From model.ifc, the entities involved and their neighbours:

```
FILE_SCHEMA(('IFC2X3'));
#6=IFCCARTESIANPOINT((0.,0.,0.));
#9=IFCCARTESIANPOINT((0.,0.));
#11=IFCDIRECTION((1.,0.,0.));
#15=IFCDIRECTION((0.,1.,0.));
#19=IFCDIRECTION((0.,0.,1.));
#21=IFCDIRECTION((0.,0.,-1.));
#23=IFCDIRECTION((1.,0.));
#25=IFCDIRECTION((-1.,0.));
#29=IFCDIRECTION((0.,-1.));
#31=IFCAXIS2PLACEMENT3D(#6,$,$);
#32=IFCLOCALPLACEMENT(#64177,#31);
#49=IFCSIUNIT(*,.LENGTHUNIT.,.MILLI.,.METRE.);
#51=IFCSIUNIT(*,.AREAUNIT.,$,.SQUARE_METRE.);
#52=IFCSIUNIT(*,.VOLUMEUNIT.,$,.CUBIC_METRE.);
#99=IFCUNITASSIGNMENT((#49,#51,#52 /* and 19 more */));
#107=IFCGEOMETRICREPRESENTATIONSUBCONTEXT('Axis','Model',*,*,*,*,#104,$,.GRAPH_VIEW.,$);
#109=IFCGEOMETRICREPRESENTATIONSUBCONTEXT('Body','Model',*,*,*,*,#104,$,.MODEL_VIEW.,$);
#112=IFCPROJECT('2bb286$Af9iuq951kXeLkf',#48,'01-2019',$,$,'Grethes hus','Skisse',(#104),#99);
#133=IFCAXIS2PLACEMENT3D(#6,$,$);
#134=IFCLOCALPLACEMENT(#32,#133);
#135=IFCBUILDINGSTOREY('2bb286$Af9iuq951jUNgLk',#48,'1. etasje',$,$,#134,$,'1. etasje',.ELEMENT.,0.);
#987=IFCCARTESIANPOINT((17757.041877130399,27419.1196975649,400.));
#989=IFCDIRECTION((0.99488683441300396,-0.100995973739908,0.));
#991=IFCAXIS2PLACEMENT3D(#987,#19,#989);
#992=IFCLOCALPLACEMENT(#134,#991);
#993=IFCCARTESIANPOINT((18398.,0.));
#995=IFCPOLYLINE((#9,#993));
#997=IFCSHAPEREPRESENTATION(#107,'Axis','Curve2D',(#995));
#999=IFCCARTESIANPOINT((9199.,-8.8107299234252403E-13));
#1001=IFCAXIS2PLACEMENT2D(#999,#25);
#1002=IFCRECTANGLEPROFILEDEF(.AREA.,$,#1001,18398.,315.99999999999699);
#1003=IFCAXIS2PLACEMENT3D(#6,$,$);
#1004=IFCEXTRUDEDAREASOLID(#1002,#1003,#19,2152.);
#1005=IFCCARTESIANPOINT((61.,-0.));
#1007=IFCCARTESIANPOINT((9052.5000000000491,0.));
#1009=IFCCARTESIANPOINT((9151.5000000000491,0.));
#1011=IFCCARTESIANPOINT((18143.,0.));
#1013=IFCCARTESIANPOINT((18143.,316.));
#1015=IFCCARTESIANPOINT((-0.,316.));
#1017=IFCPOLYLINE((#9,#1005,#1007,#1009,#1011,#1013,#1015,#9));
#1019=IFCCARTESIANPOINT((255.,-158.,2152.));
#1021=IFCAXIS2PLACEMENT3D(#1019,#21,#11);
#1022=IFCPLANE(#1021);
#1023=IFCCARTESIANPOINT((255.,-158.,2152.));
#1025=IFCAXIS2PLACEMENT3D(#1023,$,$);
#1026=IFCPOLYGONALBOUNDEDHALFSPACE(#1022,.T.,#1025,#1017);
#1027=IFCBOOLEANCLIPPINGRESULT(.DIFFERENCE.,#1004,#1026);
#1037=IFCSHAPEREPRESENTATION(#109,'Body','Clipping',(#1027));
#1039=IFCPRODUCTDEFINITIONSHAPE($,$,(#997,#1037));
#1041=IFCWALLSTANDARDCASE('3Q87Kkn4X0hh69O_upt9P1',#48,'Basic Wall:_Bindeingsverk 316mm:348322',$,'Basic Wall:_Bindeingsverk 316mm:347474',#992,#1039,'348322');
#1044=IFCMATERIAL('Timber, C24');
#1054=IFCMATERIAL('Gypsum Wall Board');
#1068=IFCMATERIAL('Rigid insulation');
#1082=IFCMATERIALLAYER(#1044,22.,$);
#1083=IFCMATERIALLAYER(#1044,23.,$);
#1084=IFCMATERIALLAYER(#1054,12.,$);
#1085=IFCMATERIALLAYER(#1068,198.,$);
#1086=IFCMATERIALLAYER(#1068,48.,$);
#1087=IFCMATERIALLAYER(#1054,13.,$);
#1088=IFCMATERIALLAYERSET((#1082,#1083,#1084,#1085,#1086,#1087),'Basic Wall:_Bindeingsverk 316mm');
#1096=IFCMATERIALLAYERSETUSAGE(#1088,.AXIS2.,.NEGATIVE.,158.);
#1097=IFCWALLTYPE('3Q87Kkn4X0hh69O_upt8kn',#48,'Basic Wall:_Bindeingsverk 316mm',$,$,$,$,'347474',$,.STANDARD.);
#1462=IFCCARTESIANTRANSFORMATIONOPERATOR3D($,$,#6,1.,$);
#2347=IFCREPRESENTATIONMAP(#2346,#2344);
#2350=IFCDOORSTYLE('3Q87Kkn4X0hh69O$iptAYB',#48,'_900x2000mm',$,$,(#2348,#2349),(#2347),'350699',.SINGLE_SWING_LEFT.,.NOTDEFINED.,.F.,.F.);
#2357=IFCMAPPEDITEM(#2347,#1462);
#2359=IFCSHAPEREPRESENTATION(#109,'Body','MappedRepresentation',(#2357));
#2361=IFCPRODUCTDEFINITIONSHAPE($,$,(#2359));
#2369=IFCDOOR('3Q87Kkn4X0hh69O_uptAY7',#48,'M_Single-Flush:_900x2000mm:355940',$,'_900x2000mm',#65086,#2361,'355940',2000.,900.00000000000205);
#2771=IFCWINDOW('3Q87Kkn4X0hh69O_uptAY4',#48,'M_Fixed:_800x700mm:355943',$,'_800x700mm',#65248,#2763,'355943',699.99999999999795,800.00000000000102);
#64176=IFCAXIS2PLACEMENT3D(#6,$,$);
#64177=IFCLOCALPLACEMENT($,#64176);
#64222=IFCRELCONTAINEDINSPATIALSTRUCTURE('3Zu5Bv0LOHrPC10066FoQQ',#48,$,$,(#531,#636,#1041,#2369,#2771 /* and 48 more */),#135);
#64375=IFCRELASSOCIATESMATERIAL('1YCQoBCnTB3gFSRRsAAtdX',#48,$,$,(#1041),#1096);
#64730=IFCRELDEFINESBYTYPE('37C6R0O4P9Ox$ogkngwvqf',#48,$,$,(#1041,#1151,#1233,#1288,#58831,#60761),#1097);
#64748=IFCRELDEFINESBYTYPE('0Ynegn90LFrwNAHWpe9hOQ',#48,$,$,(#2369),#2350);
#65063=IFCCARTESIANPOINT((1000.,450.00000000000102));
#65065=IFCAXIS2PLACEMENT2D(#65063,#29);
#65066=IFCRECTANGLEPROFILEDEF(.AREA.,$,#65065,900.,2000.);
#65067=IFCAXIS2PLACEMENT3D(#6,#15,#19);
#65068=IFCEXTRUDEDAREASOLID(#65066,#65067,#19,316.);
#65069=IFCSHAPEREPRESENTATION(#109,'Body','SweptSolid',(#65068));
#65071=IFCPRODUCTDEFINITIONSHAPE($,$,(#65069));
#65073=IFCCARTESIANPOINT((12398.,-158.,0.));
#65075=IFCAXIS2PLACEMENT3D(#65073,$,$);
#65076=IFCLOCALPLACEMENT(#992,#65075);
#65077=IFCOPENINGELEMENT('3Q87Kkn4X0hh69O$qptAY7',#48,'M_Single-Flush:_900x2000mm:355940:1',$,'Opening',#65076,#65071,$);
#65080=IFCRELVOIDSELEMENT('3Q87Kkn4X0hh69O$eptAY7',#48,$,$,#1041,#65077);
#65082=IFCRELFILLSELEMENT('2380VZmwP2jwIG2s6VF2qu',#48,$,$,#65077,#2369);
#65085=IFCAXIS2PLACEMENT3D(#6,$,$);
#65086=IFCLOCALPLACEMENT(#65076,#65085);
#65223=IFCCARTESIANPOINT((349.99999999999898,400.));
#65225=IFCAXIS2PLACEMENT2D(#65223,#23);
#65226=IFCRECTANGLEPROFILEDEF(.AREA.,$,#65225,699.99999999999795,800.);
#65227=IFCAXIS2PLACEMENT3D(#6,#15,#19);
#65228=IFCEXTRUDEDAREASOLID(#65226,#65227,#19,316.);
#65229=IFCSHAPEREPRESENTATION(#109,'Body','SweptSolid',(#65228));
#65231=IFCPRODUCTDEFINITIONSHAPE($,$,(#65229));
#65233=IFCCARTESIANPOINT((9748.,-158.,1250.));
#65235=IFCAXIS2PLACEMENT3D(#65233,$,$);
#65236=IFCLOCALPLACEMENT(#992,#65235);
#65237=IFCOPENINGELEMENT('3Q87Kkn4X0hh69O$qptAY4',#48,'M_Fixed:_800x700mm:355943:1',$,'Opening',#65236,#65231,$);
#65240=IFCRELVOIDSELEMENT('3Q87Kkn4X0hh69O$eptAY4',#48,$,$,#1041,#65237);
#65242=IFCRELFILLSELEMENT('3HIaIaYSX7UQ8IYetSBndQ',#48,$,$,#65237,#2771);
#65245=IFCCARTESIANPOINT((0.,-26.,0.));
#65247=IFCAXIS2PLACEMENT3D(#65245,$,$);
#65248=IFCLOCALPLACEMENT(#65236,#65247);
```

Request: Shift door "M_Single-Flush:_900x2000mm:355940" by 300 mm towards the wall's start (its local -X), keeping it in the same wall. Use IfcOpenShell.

```python
import ifcopenshell
import ifcopenshell.api.geometry
import ifcopenshell.util.placement
import ifcopenshell.util.unit

model = ifcopenshell.open("model.ifc")
unit_scale = ifcopenshell.util.unit.calculate_unit_scale(model)

door = model.by_id(2369)
opening = door.FillsVoids[0].RelatingOpeningElement
wall = opening.VoidsElements[0].RelatingBuildingElement

wall_matrix = ifcopenshell.util.placement.get_local_placement(wall.ObjectPlacement)
shift = wall_matrix[:3, 0] * -0.3 / unit_scale
before = ifcopenshell.util.placement.get_local_placement(door.ObjectPlacement)[:3, 3].copy()

# The door is placed relative to its opening, so it follows when the opening moves.
matrix = ifcopenshell.util.placement.get_local_placement(opening.ObjectPlacement)
matrix[:3, 3] += shift
ifcopenshell.api.geometry.edit_object_placement(
    model, product=opening, matrix=matrix, is_si=False, should_transform_children=True
)

after = ifcopenshell.util.placement.get_local_placement(door.ObjectPlacement)[:3, 3]
print("door moved by", (after - before).round(3) + 0.0)

model.write("model_updated.ifc")
```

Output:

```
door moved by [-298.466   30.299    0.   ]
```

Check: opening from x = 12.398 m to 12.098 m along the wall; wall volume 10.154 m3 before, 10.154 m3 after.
